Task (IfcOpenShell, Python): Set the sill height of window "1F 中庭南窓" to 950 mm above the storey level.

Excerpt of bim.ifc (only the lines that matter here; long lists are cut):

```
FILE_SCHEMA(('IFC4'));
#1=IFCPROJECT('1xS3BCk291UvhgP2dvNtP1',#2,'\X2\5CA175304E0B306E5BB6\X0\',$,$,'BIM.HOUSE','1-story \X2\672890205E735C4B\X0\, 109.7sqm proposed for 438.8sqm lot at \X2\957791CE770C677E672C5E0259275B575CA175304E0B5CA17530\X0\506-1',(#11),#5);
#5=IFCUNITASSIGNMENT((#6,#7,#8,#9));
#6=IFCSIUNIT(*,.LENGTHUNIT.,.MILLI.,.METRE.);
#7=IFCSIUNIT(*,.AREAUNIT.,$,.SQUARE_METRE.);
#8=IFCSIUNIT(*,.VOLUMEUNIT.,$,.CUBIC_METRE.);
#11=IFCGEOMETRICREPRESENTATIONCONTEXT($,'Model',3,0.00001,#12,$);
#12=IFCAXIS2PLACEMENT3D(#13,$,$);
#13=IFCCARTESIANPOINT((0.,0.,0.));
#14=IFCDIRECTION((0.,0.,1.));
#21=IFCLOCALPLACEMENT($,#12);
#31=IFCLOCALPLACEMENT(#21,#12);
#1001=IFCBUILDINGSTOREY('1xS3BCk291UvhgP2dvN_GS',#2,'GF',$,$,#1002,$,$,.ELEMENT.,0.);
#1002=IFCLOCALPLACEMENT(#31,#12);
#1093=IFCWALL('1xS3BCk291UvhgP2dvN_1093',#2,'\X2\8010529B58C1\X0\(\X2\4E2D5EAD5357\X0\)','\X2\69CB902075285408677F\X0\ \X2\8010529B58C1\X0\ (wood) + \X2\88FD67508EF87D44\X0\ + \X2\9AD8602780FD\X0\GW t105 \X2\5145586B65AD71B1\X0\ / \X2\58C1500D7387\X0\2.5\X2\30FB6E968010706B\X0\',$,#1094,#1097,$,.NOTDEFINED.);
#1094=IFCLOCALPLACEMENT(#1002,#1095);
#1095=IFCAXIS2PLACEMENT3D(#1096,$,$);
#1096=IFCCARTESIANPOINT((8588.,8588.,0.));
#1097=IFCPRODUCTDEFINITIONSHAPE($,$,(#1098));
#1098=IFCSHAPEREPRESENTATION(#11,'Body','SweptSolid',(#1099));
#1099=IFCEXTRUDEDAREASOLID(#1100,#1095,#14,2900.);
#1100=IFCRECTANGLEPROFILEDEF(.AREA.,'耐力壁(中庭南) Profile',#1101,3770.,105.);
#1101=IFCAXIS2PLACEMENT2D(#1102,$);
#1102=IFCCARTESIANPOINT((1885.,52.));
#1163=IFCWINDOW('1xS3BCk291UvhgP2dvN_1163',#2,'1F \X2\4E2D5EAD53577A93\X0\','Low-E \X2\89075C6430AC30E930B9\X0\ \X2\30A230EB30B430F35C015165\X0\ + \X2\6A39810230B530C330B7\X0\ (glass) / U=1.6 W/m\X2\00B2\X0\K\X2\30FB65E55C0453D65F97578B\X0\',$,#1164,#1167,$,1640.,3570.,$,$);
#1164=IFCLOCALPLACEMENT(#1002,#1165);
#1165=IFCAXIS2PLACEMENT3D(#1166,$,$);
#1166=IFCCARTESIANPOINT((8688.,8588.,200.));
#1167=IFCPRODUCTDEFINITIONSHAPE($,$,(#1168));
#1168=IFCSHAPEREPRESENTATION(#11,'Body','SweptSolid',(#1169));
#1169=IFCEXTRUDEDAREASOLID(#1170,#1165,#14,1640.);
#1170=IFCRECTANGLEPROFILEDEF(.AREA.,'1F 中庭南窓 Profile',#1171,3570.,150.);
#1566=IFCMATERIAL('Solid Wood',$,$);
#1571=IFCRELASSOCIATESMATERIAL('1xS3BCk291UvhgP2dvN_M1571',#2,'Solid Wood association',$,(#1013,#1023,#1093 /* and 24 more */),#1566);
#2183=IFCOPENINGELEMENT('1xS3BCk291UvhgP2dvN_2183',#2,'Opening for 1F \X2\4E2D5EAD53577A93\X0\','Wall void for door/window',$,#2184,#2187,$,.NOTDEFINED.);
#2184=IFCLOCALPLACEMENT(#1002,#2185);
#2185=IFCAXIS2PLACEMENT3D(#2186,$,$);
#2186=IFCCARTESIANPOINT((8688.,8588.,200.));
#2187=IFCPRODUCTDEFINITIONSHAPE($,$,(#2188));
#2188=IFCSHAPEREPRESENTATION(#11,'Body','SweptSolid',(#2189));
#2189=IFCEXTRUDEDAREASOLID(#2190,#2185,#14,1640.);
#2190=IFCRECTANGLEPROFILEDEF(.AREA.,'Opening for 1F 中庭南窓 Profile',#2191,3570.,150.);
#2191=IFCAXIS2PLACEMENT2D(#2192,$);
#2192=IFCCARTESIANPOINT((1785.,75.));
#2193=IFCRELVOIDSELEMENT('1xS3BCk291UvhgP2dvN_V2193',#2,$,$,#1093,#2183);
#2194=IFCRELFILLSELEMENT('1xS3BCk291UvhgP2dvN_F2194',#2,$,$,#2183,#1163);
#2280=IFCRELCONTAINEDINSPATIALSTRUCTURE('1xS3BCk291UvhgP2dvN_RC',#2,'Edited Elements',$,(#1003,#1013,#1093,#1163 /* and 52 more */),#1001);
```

```python
import numpy as np
import ifcopenshell
import ifcopenshell.api.geometry
import ifcopenshell.geom
import ifcopenshell.util.element
import ifcopenshell.util.placement
import ifcopenshell.util.shape
import ifcopenshell.util.unit

model = ifcopenshell.open("bim.ifc")
unit_scale = ifcopenshell.util.unit.calculate_unit_scale(model)

window = model.by_guid("1xS3BCk291UvhgP2dvN_1163")
opening = window.FillsVoids[0].RelatingOpeningElement
storey = ifcopenshell.util.element.get_container(window, ifc_class="IfcBuildingStorey")
level = ifcopenshell.util.placement.get_local_placement(storey.ObjectPlacement)[2, 3]

# The opening's origin need not be at the sill, so measure its lowest point.
shape = ifcopenshell.geom.create_shape(ifcopenshell.geom.settings(), opening)
bottom = ifcopenshell.util.shape.get_shape_bottom_elevation(shape, shape.geometry) / unit_scale
dz = level + 950.0 - bottom

shift = np.array([0.0, 0.0, dz])
# The window is not placed relative to its opening, so move both.
for product in (opening, window):
    matrix = ifcopenshell.util.placement.get_local_placement(product.ObjectPlacement)
    matrix[:3, 3] += shift
    ifcopenshell.api.geometry.edit_object_placement(model, product=product, matrix=matrix, is_si=False)

print(f"moved by {dz * unit_scale:+.3f} m")

model.write("bim_v2.ifc")
```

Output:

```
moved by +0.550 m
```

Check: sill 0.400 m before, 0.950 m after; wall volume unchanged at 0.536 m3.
